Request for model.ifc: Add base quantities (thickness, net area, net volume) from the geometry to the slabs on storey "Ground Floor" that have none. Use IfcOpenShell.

First a look at what the model holds.

```python
import ifcopenshell
import ifcopenshell.util.element
import ifcopenshell.util.unit

model = ifcopenshell.open("model.ifc")
print(model.schema)
for unit_type in ("LENGTHUNIT", "AREAUNIT", "VOLUMEUNIT"):
    print(unit_type, ifcopenshell.util.unit.calculate_unit_scale(model, unit_type))
storey = next(s for s in model.by_type("IfcBuildingStorey") if s.Name == "Ground Floor")
slabs = [e for e in ifcopenshell.util.element.get_decomposition(storey) if e.is_a("IfcSlab")]
for e in sorted(slabs, key=lambda e: e.id()):
    print(e.id(), e.is_a(), e.Name, list(ifcopenshell.util.element.get_psets(e, qtos_only=True)), sep=" | ")
```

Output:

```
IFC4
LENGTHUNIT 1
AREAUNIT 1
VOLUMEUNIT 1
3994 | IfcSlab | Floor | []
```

```python
import ifcopenshell
import ifcopenshell.api.pset
import ifcopenshell.geom
import ifcopenshell.util.element
import ifcopenshell.util.shape
import ifcopenshell.util.unit

model = ifcopenshell.open("model.ifc")
unit_scale = ifcopenshell.util.unit.calculate_unit_scale(model)
area_scale = ifcopenshell.util.unit.calculate_unit_scale(model, "AREAUNIT")
volume_scale = ifcopenshell.util.unit.calculate_unit_scale(model, "VOLUMEUNIT")
settings = ifcopenshell.geom.settings()

storey = next(s for s in model.by_type("IfcBuildingStorey") if s.Name == "Ground Floor")
slabs = [e for e in ifcopenshell.util.element.get_decomposition(storey) if e.is_a("IfcSlab")]

for e in sorted(slabs, key=lambda e: e.id()):
    if ifcopenshell.util.element.get_psets(e, qtos_only=True, should_inherit=False):
        continue
    # Geometry comes back in metres, in the element's own axes.
    shape = ifcopenshell.geom.create_shape(settings, e)
    values = {
        "Width": ifcopenshell.util.shape.get_z(shape.geometry) / unit_scale,
        "NetArea": ifcopenshell.util.shape.get_footprint_area(shape.geometry) / area_scale,
        "NetVolume": ifcopenshell.util.shape.get_volume(shape.geometry) / volume_scale,
    }
    qto = ifcopenshell.api.pset.add_qto(model, product=e, name="Qto_SlabBaseQuantities")
    ifcopenshell.api.pset.edit_qto(model, qto=qto, properties=values)
    print(e.id(), {k: round(v, 3) for k, v in values.items()})

model.write("model_edited.ifc")
```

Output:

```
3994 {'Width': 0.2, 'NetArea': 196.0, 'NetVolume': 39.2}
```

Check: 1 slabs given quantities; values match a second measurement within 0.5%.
